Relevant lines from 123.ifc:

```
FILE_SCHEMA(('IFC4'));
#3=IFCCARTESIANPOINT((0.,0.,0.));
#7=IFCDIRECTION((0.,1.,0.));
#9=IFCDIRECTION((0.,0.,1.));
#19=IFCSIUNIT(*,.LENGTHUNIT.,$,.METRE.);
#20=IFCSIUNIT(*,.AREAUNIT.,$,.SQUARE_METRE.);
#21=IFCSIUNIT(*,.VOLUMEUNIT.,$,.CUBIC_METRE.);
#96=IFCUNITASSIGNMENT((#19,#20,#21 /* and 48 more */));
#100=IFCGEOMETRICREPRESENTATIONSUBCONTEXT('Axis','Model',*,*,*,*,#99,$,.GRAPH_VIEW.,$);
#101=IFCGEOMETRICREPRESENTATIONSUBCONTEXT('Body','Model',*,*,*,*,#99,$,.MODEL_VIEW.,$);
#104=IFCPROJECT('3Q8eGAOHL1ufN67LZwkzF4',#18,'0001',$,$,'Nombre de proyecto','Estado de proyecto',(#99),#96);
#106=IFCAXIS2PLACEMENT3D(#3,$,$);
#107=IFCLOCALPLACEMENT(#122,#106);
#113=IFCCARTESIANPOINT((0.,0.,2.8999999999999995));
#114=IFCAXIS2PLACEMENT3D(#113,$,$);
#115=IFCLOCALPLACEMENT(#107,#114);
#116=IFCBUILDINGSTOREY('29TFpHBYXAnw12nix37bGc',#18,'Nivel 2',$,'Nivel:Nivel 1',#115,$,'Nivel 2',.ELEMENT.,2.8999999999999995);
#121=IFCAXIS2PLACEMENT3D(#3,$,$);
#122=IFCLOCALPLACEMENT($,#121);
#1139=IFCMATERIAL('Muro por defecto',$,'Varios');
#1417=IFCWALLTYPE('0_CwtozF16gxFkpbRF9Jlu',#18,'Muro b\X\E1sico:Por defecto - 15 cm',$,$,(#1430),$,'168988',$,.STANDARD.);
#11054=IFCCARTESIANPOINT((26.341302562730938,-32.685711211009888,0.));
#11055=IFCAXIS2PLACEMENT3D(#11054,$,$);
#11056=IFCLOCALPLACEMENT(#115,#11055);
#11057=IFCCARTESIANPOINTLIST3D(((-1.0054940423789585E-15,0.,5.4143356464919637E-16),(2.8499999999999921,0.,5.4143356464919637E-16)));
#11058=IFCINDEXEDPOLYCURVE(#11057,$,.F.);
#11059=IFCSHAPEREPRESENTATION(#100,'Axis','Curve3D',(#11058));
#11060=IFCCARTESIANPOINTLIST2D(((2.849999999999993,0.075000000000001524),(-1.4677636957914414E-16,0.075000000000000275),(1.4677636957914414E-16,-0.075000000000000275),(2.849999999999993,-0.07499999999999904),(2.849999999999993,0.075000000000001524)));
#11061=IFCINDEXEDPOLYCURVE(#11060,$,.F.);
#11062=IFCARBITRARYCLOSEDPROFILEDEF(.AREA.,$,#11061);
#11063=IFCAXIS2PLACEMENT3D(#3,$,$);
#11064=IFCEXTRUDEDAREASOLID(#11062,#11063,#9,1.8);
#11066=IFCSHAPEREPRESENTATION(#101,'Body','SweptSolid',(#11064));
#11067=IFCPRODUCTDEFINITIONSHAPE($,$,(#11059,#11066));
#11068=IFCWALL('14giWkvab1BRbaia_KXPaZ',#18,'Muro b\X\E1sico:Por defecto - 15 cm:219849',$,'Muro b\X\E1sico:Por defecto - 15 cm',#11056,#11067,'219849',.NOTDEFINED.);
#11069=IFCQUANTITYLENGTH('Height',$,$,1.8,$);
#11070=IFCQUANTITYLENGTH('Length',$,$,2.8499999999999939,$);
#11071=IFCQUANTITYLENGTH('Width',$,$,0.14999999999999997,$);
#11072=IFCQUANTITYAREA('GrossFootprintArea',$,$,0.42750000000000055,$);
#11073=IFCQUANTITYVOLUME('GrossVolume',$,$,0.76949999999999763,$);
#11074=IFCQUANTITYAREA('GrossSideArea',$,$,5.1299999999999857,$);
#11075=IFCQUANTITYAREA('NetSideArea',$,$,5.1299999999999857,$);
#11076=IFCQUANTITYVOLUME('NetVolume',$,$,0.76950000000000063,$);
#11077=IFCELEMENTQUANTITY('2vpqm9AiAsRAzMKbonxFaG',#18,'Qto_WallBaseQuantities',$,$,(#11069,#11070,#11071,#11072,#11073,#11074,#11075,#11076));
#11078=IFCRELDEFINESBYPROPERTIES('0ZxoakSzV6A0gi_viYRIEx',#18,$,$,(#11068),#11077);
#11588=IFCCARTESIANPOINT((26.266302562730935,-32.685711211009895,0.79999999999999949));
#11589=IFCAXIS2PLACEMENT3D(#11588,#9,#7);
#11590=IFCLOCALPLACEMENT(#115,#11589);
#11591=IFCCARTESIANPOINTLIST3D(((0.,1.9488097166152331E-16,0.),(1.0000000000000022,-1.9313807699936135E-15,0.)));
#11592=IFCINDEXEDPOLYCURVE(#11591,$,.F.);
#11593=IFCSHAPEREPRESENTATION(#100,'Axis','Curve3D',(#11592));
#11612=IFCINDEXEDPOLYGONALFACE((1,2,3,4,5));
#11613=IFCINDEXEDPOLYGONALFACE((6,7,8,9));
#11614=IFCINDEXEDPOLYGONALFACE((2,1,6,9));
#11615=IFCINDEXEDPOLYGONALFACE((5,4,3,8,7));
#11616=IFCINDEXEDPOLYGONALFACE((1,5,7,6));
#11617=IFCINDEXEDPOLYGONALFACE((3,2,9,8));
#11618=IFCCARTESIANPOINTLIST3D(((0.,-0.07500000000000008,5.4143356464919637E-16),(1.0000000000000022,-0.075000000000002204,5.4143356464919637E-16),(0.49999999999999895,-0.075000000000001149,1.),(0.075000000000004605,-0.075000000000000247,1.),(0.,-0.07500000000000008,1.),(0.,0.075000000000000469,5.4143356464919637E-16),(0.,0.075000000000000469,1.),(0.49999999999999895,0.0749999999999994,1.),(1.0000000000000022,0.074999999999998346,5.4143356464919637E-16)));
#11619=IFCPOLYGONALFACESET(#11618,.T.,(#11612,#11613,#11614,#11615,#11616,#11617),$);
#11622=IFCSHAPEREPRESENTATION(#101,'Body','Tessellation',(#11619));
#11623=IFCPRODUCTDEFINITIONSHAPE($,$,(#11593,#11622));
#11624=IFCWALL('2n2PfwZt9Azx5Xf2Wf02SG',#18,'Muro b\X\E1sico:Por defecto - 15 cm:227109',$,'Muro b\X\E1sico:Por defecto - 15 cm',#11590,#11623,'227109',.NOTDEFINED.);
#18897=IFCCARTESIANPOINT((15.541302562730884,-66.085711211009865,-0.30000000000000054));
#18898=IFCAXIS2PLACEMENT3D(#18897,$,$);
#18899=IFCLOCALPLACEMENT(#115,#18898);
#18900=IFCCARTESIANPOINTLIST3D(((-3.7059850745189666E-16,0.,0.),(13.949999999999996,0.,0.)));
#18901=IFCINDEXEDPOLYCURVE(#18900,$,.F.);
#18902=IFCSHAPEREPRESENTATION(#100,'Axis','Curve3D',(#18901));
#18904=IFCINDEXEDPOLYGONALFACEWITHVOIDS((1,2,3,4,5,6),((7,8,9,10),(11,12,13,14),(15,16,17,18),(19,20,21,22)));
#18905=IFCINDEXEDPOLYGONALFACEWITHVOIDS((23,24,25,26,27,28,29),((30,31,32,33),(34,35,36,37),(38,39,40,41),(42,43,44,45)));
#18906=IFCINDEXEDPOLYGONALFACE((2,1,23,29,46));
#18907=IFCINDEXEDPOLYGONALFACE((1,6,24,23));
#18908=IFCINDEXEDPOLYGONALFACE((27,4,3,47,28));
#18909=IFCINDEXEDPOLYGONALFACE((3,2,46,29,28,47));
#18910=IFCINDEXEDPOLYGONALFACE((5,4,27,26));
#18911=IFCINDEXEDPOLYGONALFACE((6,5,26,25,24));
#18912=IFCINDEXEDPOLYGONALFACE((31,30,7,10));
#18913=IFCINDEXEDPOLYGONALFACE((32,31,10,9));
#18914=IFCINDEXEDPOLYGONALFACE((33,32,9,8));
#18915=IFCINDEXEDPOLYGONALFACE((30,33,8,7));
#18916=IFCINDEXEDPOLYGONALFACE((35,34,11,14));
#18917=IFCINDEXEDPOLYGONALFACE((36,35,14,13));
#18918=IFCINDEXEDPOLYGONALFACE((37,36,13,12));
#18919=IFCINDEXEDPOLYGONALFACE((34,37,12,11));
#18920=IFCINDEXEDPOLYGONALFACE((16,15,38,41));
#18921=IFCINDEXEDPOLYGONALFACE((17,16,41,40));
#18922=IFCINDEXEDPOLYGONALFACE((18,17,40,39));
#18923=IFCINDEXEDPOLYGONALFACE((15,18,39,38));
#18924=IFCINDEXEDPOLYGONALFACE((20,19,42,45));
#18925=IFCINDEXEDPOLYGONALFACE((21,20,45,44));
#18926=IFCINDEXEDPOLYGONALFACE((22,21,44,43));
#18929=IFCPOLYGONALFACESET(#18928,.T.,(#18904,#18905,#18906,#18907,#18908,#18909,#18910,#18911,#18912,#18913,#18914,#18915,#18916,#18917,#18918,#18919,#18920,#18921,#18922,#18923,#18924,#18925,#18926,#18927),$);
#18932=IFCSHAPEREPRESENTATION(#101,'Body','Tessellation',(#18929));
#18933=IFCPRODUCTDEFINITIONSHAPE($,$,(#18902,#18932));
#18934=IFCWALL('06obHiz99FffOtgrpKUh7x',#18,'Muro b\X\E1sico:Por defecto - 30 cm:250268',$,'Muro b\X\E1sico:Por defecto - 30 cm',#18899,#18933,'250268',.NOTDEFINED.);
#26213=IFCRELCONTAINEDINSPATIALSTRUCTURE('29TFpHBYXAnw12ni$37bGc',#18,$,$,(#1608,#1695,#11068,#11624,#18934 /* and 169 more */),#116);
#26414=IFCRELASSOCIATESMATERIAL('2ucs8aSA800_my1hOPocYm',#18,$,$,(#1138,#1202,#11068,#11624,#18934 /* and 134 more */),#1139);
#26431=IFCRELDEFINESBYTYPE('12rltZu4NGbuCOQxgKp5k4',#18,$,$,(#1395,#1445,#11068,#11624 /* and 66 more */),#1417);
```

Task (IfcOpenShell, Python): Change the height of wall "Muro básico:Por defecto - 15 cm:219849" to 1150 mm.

```python
import ifcopenshell
import ifcopenshell.api.pset
import ifcopenshell.geom
import ifcopenshell.util.element
import ifcopenshell.util.representation
import ifcopenshell.util.shape
import ifcopenshell.util.unit

model = ifcopenshell.open("123.ifc")
unit_scale = ifcopenshell.util.unit.calculate_unit_scale(model)
area_scale = ifcopenshell.util.unit.calculate_unit_scale(model, "AREAUNIT")
volume_scale = ifcopenshell.util.unit.calculate_unit_scale(model, "VOLUMEUNIT")
settings = ifcopenshell.geom.settings()


def volume(element):
    """Net volume in cubic metres, openings subtracted."""
    shape = ifcopenshell.geom.create_shape(settings, element)
    return ifcopenshell.util.shape.get_volume(shape.geometry)


wall = model.by_guid("14giWkvab1BRbaia_KXPaZ")
before = volume(wall)

body = ifcopenshell.util.representation.get_representation(wall, "Model", "Body")
solid = body.Items[0]
old_height = solid.Depth
solid.Depth = 1.15 / unit_scale
after = volume(wall)
thickness = 0.15  # wall thickness in metres

# Update the stored height, areas and volumes.
qto = model.by_id(ifcopenshell.util.element.get_pset(wall, "Qto_WallBaseQuantities", should_inherit=False)["id"])
ifcopenshell.api.pset.edit_qto(model, qto=qto, properties={
    "Height": solid.Depth,
    "GrossVolume": ifcopenshell.util.element.get_pset(wall, "Qto_WallBaseQuantities", "GrossVolume") * solid.Depth / old_height,
    "GrossSideArea": ifcopenshell.util.element.get_pset(wall, "Qto_WallBaseQuantities", "GrossSideArea") * solid.Depth / old_height,
    "NetSideArea": after / thickness / area_scale,
    "NetVolume": after / volume_scale,
})

print(f"height {old_height:g} -> {solid.Depth:g}, volume {before:.3f} -> {after:.3f} m3")

model.write("123_v2.ifc")
```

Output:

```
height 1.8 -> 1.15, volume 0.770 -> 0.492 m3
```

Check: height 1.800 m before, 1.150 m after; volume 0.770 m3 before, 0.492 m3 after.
